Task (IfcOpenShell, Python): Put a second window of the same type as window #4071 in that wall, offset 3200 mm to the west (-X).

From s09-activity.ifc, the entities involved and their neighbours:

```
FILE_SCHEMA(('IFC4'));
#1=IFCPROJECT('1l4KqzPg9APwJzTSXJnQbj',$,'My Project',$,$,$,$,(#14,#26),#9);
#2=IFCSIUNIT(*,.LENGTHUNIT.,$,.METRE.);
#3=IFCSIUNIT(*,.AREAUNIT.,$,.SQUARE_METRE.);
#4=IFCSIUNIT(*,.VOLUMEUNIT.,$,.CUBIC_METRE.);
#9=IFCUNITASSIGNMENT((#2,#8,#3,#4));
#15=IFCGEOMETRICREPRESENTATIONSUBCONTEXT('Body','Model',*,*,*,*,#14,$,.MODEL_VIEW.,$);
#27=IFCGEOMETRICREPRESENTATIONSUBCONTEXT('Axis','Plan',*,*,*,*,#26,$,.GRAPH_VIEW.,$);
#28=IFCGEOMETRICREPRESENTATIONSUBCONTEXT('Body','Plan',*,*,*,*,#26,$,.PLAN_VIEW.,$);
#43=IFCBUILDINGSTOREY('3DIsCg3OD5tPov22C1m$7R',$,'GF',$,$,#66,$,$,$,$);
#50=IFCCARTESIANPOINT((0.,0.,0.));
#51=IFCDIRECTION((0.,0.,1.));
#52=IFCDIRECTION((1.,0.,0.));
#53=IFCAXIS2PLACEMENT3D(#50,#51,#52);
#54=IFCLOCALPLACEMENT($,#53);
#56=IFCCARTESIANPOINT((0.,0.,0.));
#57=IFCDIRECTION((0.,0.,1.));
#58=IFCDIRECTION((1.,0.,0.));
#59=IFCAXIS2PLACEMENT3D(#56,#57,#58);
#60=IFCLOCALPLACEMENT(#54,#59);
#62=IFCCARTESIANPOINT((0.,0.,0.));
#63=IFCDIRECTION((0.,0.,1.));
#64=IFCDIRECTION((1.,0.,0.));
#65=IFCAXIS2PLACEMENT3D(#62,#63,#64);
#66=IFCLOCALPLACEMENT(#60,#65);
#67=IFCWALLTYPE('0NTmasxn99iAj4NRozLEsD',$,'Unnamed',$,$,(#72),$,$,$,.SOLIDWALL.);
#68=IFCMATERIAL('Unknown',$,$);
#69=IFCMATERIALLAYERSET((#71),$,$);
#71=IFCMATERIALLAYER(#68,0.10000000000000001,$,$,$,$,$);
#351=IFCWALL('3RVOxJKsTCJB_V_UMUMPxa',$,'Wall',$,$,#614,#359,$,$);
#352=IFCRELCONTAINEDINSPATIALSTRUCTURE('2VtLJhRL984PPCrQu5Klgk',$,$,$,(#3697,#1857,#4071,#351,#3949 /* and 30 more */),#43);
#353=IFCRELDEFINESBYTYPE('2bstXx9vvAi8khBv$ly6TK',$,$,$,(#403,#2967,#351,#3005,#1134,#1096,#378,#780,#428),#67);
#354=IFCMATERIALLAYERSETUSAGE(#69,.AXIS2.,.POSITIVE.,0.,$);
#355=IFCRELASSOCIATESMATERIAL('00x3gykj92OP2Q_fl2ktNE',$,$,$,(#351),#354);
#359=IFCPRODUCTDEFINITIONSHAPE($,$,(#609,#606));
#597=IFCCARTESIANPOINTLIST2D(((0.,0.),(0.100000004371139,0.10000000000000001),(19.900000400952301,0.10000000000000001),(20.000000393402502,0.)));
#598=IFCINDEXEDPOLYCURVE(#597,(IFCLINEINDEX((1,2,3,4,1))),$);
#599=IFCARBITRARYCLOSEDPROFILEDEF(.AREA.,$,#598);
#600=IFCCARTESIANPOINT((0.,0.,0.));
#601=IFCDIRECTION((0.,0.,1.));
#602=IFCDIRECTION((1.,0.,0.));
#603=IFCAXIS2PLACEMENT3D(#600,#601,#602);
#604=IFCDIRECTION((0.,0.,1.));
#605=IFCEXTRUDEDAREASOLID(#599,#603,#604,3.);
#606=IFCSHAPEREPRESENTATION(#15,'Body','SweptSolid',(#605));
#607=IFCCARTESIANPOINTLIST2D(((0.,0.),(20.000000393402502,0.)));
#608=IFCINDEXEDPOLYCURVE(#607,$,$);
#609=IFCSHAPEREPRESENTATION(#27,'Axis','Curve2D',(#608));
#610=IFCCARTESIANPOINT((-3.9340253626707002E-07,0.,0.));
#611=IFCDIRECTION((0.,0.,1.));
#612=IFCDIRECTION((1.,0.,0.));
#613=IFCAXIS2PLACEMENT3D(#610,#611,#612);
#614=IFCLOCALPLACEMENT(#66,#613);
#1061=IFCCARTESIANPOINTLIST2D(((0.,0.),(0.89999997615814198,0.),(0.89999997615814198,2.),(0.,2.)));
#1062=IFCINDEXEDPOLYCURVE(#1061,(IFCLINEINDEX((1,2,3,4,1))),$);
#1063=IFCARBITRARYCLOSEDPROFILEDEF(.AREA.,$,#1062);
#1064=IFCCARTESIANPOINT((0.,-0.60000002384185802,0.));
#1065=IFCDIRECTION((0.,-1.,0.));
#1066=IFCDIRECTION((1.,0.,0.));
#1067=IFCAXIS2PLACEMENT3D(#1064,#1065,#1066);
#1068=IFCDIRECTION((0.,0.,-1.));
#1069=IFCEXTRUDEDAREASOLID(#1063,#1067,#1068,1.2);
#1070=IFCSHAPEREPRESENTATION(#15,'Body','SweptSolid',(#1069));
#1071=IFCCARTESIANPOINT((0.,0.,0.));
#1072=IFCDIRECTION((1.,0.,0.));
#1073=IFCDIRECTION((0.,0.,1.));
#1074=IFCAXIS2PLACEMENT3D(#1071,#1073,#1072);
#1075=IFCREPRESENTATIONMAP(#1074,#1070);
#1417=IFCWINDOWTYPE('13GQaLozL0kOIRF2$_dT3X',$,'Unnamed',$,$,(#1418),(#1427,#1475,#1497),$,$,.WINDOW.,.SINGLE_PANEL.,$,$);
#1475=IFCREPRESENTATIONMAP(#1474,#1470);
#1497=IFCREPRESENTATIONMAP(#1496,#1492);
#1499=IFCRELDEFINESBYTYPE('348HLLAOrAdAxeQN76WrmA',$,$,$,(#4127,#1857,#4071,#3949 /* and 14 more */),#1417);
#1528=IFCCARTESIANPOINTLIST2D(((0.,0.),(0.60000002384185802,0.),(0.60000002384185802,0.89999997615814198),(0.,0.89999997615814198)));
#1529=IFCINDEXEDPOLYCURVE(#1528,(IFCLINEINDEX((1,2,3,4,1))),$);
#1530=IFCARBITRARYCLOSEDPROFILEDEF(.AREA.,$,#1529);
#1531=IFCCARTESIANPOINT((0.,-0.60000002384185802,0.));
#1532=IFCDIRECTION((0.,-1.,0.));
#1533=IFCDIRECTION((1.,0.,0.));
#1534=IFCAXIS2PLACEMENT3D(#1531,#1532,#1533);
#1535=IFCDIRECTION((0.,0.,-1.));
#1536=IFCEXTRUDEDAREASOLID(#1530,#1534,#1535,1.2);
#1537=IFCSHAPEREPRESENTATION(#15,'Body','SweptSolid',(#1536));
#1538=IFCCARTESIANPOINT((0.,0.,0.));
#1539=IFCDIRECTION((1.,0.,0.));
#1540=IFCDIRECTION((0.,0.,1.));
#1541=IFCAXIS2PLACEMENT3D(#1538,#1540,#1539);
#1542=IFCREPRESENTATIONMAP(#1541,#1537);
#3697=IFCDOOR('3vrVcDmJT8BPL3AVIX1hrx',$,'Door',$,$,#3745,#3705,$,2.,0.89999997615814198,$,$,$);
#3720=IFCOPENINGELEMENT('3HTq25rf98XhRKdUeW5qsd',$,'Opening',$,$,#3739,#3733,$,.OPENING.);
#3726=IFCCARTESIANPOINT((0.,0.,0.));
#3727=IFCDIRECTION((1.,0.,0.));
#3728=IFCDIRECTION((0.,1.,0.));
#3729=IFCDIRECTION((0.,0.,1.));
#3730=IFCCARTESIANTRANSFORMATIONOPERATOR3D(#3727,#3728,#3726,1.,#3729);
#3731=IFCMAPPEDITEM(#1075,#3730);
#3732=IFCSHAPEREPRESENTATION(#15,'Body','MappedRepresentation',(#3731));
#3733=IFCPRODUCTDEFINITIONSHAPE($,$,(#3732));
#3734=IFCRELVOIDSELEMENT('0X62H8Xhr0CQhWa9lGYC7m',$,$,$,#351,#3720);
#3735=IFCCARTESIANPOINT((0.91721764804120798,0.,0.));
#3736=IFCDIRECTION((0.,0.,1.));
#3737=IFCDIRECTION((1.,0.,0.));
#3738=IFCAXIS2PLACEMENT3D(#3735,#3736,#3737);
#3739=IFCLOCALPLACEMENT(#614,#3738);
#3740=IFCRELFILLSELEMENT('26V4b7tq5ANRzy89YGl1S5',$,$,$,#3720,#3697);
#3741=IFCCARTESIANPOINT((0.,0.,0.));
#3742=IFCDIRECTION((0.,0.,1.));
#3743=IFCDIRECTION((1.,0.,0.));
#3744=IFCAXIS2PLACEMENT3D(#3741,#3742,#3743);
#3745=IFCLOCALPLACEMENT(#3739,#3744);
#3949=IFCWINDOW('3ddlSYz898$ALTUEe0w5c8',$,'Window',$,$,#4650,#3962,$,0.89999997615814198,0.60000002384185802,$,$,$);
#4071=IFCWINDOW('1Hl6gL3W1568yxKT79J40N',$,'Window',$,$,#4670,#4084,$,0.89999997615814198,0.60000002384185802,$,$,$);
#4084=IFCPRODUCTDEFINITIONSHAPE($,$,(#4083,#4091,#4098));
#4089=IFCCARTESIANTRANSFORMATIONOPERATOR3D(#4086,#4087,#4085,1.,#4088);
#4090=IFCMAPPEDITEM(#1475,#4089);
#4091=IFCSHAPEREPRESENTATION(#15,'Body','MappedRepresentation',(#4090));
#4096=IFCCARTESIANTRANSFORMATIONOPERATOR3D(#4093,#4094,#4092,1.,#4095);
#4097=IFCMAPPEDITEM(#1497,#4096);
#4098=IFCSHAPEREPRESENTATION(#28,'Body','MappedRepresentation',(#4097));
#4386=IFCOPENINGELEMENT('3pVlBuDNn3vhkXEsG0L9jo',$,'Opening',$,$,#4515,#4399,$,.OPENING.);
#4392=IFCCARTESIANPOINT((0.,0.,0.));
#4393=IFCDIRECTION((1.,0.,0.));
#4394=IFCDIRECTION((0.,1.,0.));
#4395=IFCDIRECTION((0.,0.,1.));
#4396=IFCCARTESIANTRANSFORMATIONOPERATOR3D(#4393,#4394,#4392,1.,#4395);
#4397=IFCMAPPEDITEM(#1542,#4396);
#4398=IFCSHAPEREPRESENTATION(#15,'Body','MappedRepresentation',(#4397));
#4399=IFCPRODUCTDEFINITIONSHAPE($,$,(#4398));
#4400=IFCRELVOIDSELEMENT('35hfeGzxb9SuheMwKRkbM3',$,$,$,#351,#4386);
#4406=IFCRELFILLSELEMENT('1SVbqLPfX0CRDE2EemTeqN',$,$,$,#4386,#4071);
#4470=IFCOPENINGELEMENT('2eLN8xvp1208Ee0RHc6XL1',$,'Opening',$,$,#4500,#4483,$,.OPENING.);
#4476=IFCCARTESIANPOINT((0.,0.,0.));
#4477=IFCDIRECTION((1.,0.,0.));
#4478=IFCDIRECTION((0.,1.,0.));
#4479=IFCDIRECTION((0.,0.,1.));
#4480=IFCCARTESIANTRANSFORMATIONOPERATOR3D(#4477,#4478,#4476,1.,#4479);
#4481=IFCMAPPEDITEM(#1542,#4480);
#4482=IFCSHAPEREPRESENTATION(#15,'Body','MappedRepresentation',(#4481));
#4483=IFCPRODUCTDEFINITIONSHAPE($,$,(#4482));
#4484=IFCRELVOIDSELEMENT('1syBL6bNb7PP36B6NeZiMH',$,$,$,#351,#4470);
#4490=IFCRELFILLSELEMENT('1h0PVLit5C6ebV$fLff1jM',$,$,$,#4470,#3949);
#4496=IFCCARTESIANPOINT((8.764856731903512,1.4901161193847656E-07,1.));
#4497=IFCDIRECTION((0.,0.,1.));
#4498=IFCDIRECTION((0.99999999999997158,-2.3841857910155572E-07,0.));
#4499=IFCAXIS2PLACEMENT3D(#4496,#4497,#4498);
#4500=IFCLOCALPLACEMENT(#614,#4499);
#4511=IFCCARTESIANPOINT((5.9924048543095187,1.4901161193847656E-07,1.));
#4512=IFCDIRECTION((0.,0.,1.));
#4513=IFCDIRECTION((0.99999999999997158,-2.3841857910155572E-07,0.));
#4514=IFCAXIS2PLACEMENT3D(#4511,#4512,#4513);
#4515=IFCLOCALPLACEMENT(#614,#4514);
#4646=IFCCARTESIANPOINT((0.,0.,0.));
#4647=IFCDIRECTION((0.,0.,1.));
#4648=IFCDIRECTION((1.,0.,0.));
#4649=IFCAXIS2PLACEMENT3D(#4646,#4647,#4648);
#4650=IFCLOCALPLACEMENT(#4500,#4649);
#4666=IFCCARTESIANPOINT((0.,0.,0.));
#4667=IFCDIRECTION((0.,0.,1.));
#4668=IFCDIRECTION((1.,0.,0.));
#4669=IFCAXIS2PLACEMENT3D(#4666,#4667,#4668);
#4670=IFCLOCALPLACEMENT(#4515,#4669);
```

```python
import ifcopenshell
import ifcopenshell.api.feature
import ifcopenshell.api.geometry
import ifcopenshell.api.root
import ifcopenshell.geom
import ifcopenshell.util.element
import ifcopenshell.util.placement
import ifcopenshell.util.shape

model = ifcopenshell.open("s09-activity.ifc")
settings = ifcopenshell.geom.settings()


def volume(element):
    """Net volume in cubic metres, openings subtracted."""
    shape = ifcopenshell.geom.create_shape(settings, element)
    return ifcopenshell.util.shape.get_volume(shape.geometry)


window = model.by_id(4071)
opening = window.FillsVoids[0].RelatingOpeningElement
wall = opening.VoidsElements[0].RelatingBuildingElement
before = volume(wall)
shift = ifcopenshell.util.placement.get_local_placement(wall.ObjectPlacement)[:3, 0] * -3.2

# copy_class copies the void relationship, type, container and properties, but no geometry.
new_opening = ifcopenshell.api.root.copy_class(model, product=opening)
new_opening.Representation = ifcopenshell.util.element.copy_deep(
    model, opening.Representation, exclude=["IfcGeometricRepresentationContext", "IfcRepresentationMap"]
)
new_window = ifcopenshell.api.root.copy_class(model, product=window)
new_window.Representation = ifcopenshell.util.element.copy_deep(
    model, window.Representation, exclude=["IfcGeometricRepresentationContext", "IfcRepresentationMap"]
)
ifcopenshell.api.feature.add_filling(model, opening=new_opening, element=new_window)

for old, new in ((opening, new_opening), (window, new_window)):
    matrix = ifcopenshell.util.placement.get_local_placement(old.ObjectPlacement)
    matrix[:3, 3] += shift
    ifcopenshell.api.geometry.edit_object_placement(model, product=new, matrix=matrix, is_si=False)

after = volume(wall)

print(f"wall volume {before:.3f} -> {after:.3f} m3")

model.write("s09-activity_v2.ifc")
```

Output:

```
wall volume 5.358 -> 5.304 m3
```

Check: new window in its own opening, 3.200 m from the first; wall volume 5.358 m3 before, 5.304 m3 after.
